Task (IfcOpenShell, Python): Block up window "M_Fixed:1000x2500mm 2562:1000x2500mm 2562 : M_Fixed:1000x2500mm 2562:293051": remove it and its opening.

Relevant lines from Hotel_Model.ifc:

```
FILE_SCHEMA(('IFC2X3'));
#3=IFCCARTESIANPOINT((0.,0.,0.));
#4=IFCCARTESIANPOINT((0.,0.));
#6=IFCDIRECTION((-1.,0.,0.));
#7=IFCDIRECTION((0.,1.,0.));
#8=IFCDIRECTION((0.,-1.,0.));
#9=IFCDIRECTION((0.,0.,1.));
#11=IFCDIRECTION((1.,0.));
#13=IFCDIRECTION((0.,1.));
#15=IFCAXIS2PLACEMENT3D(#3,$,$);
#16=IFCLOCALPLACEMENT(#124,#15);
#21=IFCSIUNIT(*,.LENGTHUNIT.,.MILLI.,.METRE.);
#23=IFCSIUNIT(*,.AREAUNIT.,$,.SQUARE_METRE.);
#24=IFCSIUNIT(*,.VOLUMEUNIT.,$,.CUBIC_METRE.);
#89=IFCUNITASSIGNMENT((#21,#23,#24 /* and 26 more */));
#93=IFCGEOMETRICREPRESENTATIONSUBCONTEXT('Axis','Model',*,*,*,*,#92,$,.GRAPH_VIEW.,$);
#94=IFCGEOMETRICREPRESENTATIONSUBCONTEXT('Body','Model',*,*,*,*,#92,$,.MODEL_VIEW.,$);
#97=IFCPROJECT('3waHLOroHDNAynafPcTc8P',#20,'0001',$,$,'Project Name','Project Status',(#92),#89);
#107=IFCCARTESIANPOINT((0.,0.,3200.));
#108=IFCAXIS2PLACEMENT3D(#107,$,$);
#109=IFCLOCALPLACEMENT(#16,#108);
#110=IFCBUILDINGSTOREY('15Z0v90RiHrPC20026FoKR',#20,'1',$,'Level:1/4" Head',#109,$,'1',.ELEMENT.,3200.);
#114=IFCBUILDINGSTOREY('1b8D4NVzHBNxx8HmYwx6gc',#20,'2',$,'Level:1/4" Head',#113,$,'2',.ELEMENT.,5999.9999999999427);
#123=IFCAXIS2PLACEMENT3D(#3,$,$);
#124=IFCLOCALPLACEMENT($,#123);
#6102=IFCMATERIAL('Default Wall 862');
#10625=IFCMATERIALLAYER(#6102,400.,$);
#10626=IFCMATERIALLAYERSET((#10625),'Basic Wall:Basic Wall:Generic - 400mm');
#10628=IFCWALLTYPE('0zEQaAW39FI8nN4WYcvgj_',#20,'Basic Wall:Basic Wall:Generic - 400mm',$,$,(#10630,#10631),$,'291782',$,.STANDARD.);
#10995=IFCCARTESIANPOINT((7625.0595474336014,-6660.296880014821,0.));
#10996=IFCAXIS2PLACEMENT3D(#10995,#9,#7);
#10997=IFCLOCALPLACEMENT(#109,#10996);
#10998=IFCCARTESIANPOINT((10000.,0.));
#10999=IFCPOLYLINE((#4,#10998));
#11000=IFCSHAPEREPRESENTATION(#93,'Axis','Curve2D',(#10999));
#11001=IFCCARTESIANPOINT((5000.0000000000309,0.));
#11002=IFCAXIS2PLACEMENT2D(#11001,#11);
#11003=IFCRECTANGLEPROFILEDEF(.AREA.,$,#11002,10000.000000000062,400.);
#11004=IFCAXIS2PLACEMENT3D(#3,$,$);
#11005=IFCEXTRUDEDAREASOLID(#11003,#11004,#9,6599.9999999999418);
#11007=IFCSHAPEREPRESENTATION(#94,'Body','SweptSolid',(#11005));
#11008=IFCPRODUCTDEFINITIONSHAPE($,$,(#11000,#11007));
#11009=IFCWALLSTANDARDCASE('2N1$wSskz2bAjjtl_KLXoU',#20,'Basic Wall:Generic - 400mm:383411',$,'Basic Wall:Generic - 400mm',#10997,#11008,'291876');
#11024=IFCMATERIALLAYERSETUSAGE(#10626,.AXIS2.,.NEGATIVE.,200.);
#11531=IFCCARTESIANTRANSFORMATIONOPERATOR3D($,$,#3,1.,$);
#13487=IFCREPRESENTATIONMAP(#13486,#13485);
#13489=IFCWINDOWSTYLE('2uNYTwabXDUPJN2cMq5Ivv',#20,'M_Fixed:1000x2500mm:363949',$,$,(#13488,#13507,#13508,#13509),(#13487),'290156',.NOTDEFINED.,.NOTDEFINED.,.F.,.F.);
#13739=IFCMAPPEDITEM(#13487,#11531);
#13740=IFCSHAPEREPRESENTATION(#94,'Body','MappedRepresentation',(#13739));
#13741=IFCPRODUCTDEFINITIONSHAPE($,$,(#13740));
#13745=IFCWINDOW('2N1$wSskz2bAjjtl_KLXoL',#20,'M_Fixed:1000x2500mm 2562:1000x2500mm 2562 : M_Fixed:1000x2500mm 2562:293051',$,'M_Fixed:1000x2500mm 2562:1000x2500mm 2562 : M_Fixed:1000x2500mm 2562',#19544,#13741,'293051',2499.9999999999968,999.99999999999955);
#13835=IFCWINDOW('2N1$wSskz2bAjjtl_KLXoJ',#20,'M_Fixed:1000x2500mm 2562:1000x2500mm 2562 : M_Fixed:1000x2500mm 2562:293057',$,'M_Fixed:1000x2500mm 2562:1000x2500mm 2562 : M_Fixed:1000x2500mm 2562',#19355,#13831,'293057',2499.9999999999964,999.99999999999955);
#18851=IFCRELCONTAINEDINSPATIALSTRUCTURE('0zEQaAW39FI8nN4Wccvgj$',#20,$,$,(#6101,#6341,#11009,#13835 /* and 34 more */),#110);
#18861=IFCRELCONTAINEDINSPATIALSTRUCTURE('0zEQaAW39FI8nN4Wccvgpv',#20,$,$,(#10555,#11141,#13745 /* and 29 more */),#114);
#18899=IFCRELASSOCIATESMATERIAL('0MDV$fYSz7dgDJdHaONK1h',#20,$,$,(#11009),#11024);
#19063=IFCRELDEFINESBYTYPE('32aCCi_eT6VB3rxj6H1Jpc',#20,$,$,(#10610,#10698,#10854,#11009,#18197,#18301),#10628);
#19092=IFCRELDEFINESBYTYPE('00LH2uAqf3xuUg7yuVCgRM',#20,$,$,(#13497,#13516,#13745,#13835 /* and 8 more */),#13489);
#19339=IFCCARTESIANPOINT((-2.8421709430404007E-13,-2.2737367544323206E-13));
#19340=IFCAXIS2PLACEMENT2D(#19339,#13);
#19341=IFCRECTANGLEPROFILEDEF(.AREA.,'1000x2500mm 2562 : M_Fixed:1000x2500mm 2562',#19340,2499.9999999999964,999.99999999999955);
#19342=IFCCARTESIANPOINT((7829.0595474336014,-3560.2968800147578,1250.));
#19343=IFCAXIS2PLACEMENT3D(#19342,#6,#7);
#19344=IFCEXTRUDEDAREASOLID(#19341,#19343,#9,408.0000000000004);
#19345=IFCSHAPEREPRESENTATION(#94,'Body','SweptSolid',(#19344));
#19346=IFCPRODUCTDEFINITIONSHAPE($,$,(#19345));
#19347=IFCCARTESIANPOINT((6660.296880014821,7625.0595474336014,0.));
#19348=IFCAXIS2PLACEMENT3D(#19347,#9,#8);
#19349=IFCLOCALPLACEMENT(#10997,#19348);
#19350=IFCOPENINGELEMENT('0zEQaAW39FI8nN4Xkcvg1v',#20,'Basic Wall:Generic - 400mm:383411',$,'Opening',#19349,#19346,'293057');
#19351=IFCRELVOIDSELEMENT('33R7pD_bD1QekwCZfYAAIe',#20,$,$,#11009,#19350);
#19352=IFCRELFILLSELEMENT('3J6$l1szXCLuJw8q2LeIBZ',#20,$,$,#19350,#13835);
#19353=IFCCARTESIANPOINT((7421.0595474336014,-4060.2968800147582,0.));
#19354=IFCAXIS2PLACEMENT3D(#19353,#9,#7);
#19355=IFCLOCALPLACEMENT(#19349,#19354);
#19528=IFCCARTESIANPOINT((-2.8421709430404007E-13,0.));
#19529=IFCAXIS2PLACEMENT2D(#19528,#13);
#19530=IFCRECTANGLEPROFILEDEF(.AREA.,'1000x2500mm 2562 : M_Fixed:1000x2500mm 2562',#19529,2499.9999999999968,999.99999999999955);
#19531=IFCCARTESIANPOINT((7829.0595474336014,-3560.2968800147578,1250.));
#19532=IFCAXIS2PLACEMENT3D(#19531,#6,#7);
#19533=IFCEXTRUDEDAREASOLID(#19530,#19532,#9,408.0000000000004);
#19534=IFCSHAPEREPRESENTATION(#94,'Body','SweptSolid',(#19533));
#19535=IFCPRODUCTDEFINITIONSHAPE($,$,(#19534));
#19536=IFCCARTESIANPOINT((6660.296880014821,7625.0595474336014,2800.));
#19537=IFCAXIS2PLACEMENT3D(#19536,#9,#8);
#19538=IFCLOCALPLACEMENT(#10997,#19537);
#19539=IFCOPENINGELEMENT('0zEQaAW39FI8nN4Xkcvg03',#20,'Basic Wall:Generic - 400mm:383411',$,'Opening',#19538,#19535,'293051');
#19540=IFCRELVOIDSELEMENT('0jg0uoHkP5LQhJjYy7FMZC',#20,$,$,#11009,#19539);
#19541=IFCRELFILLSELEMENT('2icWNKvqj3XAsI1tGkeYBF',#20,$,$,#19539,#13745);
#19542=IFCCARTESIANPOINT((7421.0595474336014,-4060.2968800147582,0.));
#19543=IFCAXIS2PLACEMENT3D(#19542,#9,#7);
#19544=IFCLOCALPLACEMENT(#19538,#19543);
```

```python
import ifcopenshell
import ifcopenshell.api.feature
import ifcopenshell.api.root
import ifcopenshell.geom
import ifcopenshell.util.shape

model = ifcopenshell.open("Hotel_Model.ifc")
settings = ifcopenshell.geom.settings()


def volume(element):
    """Net volume in cubic metres, openings subtracted."""
    shape = ifcopenshell.geom.create_shape(settings, element)
    return ifcopenshell.util.shape.get_volume(shape.geometry)


window = model.by_guid("2N1$wSskz2bAjjtl_KLXoL")
opening = window.FillsVoids[0].RelatingOpeningElement
wall = opening.VoidsElements[0].RelatingBuildingElement
before = volume(wall)

ifcopenshell.api.root.remove_product(model, product=window)
ifcopenshell.api.feature.remove_feature(model, feature=opening)

after = volume(wall)

print(f"wall volume {before:.3f} -> {after:.3f} m3")

model.write("Hotel_Model_v2.ifc")
```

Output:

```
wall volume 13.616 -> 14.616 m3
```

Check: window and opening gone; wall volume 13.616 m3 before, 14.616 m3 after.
